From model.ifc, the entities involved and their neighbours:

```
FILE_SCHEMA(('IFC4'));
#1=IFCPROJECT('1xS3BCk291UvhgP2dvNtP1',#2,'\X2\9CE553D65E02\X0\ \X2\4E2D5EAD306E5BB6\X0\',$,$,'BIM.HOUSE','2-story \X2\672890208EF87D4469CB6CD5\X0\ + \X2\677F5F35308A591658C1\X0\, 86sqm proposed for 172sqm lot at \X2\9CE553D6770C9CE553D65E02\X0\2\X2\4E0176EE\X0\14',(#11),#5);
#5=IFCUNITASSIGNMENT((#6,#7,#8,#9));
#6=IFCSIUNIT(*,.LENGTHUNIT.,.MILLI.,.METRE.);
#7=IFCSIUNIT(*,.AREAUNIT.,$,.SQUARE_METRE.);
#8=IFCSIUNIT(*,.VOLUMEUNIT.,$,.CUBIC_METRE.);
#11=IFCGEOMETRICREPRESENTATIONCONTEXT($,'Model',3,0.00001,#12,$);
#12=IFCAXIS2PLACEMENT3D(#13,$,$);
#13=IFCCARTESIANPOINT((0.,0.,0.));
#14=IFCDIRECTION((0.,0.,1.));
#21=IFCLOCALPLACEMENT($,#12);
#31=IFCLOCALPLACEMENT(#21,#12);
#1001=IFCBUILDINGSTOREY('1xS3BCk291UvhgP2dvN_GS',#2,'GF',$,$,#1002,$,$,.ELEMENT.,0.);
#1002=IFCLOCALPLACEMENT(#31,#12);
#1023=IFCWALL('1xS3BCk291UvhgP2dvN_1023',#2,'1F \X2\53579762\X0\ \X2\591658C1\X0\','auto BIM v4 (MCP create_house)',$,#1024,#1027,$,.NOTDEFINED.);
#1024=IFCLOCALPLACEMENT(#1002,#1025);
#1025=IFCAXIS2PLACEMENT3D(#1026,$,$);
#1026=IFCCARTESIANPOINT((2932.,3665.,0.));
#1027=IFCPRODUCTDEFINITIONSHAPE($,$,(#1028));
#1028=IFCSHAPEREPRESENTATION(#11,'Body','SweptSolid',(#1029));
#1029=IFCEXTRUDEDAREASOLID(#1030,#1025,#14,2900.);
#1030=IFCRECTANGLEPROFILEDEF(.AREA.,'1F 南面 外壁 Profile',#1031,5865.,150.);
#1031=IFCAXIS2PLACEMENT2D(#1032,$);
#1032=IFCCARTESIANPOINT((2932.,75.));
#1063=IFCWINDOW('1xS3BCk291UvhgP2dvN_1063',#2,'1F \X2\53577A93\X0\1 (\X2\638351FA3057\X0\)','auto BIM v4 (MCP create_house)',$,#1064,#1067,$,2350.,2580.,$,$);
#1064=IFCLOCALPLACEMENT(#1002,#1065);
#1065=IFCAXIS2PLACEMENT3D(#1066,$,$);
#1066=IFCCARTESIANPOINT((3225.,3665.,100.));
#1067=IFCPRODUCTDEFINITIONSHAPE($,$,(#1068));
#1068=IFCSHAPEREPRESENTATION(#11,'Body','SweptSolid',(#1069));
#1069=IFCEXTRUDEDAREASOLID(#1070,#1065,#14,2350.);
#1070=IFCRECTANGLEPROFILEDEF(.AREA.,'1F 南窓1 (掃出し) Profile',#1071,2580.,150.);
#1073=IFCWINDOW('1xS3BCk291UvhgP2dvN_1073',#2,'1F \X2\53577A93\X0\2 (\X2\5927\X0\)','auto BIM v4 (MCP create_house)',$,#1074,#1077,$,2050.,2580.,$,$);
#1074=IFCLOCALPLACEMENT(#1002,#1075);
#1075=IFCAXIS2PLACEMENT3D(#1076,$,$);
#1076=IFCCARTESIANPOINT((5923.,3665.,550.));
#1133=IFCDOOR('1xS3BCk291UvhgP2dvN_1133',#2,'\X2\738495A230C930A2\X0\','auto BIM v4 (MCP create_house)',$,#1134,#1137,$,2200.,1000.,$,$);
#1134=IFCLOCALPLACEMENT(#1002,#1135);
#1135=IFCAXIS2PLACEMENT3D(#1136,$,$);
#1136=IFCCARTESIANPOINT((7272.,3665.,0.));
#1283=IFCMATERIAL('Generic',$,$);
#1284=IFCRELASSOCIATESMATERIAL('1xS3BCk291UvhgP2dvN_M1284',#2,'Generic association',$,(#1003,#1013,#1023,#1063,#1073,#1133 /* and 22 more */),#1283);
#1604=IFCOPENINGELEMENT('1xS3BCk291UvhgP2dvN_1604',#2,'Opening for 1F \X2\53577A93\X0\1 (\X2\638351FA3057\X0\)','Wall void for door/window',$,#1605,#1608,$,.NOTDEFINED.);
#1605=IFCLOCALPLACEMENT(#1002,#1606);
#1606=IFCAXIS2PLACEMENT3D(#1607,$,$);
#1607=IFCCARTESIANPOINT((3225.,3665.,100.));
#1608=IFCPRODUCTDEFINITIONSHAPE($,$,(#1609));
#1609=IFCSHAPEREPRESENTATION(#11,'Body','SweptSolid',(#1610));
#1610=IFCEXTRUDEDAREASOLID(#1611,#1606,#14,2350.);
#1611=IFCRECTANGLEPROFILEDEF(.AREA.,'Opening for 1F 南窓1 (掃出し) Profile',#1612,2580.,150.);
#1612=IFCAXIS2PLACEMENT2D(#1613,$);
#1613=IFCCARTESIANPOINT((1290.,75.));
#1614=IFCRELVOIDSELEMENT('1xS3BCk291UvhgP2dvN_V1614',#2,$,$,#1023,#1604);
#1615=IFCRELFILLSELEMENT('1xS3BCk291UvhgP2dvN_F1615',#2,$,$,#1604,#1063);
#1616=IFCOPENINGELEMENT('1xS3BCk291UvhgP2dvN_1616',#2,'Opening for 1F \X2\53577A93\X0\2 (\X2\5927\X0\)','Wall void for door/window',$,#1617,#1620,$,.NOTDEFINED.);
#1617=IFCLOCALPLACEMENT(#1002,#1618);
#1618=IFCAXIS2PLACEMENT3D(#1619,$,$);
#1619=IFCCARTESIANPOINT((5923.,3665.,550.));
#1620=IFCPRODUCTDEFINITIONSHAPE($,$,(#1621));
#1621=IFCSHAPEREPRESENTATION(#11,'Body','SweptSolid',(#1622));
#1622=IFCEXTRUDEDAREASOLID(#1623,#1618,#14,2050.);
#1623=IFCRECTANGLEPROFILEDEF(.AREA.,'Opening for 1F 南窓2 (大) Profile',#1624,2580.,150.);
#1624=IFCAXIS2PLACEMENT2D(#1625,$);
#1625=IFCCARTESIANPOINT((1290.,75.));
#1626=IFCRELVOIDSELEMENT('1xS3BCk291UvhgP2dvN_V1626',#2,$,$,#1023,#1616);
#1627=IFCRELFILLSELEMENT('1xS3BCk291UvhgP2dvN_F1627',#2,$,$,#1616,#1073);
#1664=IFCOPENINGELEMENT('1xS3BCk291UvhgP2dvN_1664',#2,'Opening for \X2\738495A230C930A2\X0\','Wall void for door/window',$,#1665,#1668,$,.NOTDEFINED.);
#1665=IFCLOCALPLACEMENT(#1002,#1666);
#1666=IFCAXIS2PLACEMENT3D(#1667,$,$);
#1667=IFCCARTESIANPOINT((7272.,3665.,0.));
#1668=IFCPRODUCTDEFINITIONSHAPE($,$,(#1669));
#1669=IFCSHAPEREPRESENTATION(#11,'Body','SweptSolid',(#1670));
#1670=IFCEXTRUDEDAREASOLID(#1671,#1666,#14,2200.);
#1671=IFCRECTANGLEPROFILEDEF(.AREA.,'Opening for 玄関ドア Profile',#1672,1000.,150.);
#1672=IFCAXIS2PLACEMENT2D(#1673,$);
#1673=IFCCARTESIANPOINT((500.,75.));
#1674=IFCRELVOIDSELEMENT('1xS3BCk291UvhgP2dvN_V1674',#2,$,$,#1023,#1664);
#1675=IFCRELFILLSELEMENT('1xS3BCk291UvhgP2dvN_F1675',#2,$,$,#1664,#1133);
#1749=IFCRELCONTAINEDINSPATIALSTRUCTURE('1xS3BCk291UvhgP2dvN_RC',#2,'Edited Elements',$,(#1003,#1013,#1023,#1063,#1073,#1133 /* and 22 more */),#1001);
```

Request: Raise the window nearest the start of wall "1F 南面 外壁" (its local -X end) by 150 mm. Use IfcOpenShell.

```python
import numpy as np
import ifcopenshell
import ifcopenshell.api.geometry
import ifcopenshell.util.placement
import ifcopenshell.util.unit

model = ifcopenshell.open("model.ifc")
unit_scale = ifcopenshell.util.unit.calculate_unit_scale(model)

window = model.by_id(1063)
opening = window.FillsVoids[0].RelatingOpeningElement
dz = 0.15 / unit_scale

shift = np.array([0.0, 0.0, dz])
# The window is not placed relative to its opening, so move both.
for product in (opening, window):
    matrix = ifcopenshell.util.placement.get_local_placement(product.ObjectPlacement)
    matrix[:3, 3] += shift
    ifcopenshell.api.geometry.edit_object_placement(model, product=product, matrix=matrix, is_si=False)

print(f"moved by {dz * unit_scale:+.3f} m")

model.write("model_updated.ifc")
```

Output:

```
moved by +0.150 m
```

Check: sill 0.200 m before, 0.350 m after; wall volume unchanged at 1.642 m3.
